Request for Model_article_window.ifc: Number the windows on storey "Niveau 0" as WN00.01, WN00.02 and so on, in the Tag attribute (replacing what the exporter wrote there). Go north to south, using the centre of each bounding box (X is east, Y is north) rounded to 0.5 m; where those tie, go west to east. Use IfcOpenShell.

First a look at what the model holds.

```python
import ifcopenshell
import ifcopenshell.util.element
import ifcopenshell.util.placement

model = ifcopenshell.open("Model_article_window.ifc")
print(model.schema)
storey = next(s for s in model.by_type("IfcBuildingStorey") if s.Name == "Niveau 0")
windows = [e for e in ifcopenshell.util.element.get_decomposition(storey) if e.is_a("IfcWindow")]
for e in sorted(windows, key=lambda e: e.id()):
    origin = ifcopenshell.util.placement.get_local_placement(e.ObjectPlacement)[:3, 3]
    print(e.id(), e.Tag, e.Name, origin.round(2) + 0.0, sep=" | ")
```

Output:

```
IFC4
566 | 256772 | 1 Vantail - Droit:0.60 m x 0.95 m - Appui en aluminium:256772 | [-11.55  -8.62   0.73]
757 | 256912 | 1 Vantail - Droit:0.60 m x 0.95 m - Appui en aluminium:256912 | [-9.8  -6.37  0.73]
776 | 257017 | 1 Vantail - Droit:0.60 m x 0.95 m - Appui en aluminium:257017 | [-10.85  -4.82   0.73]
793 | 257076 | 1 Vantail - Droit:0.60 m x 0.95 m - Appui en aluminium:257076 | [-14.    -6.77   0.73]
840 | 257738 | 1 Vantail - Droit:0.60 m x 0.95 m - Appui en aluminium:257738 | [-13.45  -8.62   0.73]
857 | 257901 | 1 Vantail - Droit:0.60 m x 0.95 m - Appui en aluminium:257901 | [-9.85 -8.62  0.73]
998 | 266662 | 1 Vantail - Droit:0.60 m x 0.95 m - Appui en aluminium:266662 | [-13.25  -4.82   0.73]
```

```python
import ifcopenshell
import ifcopenshell.geom
import ifcopenshell.util.element
import ifcopenshell.util.shape

model = ifcopenshell.open("Model_article_window.ifc")
settings = ifcopenshell.geom.settings()
settings.set("use-world-coords", True)


def centre(element):
    shape = ifcopenshell.geom.create_shape(settings, element)
    return ifcopenshell.util.shape.get_bbox_centroid(shape.geometry)


storey = next(s for s in model.by_type("IfcBuildingStorey") if s.Name == "Niveau 0")
windows = [e for e in ifcopenshell.util.element.get_decomposition(storey) if e.is_a("IfcWindow")]

# Insertion points can sit at a corner or the storey origin, so sort by the geometry (in metres).
centres = {e: centre(e) for e in windows}
windows.sort(key=lambda e: (-round(centres[e][1] / 0.5), centres[e][0]))

for i, e in enumerate(windows, start=1):
    number = f"WN00.{i:02d}"
    e.Tag = number
    print(e.id(), number)

model.write("Model_article_window_v2.ifc")
```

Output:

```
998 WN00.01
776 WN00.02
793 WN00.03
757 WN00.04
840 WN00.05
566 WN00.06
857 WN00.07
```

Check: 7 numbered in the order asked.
